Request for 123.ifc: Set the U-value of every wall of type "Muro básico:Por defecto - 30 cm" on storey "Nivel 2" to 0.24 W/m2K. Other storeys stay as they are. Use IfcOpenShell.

First a look at what the model holds.

```python
import ifcopenshell
import ifcopenshell.util.element

model = ifcopenshell.open("123.ifc")
print(model.schema)
storey = next(s for s in model.by_type("IfcBuildingStorey") if s.Name == "Nivel 2")
walls = [e for e in ifcopenshell.util.element.get_decomposition(storey) if e.is_a("IfcWall")]
seen = {}
for e in walls:
    element_type = ifcopenshell.util.element.get_type(e)
    key = (element_type.Name if element_type != e and element_type else None, ifcopenshell.util.element.get_pset(e, "Pset_WallCommon", "ThermalTransmittance"))
    seen[key] = seen.get(key, 0) + 1
for (name, value), count in sorted(seen.items(), key=str):
    print(count, "x", name, "|", value)
```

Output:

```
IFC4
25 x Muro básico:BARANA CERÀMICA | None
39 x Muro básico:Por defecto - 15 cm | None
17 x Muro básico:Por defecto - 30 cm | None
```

```python
import ifcopenshell
import ifcopenshell.api.pset
import ifcopenshell.util.element

model = ifcopenshell.open("123.ifc")

storey = next(s for s in model.by_type("IfcBuildingStorey") if s.Name == "Nivel 2")
walls = [e for e in ifcopenshell.util.element.get_decomposition(storey) if e.is_a("IfcWall")]

count = 0
for e in walls:
    element_type = ifcopenshell.util.element.get_type(e)
    if element_type in (None, e) or element_type.Name != "Muro básico:Por defecto - 30 cm":
        continue
    # add_pset returns the element's existing set when there is one.
    pset = ifcopenshell.api.pset.add_pset(model, product=e, name="Pset_WallCommon")
    ifcopenshell.api.pset.edit_pset(model, pset=pset, properties={"ThermalTransmittance": 0.24})
    count += 1

print(count, "walls updated")

model.write("123-out.ifc")
```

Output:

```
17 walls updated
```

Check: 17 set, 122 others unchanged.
